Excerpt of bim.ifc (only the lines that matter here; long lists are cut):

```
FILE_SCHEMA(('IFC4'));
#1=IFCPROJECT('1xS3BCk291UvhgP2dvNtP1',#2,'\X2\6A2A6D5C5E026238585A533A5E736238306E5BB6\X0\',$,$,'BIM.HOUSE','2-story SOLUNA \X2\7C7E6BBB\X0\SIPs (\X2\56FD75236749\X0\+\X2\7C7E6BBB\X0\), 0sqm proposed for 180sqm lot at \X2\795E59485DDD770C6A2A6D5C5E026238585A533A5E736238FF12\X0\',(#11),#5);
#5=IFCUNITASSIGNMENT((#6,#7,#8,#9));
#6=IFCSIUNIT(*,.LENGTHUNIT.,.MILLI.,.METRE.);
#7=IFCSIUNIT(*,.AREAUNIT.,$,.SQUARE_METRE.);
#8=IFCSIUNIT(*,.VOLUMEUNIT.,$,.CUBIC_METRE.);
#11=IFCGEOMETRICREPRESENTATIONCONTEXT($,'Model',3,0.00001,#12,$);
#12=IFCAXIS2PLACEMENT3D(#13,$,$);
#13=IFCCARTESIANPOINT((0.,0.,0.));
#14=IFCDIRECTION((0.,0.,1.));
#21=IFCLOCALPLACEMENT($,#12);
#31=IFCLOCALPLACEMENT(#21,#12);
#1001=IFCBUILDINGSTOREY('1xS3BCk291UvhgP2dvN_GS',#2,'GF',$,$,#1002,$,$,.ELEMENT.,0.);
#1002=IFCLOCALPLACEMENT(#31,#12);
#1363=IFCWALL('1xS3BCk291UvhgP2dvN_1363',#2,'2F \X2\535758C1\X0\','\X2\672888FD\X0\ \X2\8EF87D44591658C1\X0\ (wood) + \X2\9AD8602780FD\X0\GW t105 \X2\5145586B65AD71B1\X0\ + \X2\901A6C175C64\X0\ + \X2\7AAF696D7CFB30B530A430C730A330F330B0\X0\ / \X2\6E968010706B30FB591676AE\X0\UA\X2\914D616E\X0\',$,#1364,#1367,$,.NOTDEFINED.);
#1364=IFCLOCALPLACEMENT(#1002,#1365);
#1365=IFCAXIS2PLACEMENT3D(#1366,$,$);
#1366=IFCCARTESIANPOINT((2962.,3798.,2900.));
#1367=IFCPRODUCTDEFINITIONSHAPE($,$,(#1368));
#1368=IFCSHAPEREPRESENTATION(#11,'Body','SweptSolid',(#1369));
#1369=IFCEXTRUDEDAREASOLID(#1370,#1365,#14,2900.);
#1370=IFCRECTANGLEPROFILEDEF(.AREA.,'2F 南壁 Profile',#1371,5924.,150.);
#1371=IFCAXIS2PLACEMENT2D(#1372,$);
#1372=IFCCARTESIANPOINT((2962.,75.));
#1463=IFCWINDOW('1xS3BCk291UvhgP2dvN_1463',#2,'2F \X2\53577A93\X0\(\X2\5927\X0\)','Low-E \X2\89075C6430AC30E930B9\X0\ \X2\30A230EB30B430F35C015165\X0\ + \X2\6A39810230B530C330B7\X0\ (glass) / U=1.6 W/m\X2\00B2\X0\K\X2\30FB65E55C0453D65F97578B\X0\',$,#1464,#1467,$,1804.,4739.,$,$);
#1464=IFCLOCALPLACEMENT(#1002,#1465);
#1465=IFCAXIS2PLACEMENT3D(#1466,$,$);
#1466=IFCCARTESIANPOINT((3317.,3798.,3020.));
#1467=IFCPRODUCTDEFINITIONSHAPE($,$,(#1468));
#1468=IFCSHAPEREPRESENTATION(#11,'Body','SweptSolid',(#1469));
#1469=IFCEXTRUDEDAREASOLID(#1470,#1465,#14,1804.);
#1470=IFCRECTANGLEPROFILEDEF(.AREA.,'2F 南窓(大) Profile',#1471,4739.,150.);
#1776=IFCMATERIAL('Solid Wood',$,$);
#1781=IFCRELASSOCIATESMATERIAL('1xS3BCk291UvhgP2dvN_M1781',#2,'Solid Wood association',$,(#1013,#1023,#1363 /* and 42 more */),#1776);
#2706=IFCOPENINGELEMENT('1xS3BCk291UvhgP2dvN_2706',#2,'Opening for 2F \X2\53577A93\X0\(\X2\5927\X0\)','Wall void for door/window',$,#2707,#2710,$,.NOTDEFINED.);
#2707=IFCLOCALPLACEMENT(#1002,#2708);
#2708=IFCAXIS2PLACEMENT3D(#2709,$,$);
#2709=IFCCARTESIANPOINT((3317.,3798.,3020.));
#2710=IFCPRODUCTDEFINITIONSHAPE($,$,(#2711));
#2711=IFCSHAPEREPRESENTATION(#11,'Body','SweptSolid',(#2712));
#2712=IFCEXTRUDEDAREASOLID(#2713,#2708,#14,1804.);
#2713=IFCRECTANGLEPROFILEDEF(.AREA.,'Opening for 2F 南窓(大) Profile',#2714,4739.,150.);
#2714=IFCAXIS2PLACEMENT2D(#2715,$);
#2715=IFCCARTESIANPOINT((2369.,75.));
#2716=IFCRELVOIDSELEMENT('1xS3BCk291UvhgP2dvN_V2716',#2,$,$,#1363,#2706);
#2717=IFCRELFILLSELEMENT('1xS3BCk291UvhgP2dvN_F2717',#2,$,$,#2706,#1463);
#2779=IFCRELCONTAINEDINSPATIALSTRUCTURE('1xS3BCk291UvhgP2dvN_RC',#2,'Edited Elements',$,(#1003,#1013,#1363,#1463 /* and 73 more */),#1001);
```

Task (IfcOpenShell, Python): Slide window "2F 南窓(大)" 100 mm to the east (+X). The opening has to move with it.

```python
import ifcopenshell
import ifcopenshell.api.geometry
import ifcopenshell.util.placement
import ifcopenshell.util.unit

model = ifcopenshell.open("bim.ifc")
unit_scale = ifcopenshell.util.unit.calculate_unit_scale(model)

window = model.by_guid("1xS3BCk291UvhgP2dvN_1463")
opening = window.FillsVoids[0].RelatingOpeningElement
wall = opening.VoidsElements[0].RelatingBuildingElement

wall_matrix = ifcopenshell.util.placement.get_local_placement(wall.ObjectPlacement)
shift = wall_matrix[:3, 0] * 0.1 / unit_scale
before = ifcopenshell.util.placement.get_local_placement(window.ObjectPlacement)[:3, 3].copy()

# The window is not placed relative to its opening, so move both.
for product in (opening, window):
    matrix = ifcopenshell.util.placement.get_local_placement(product.ObjectPlacement)
    matrix[:3, 3] += shift
    ifcopenshell.api.geometry.edit_object_placement(model, product=product, matrix=matrix, is_si=False)

after = ifcopenshell.util.placement.get_local_placement(window.ObjectPlacement)[:3, 3]
print("window moved by", (after - before).round(3) + 0.0)

model.write("bim_rev.ifc")
```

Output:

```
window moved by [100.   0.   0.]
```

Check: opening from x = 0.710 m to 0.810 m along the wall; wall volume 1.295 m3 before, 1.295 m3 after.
